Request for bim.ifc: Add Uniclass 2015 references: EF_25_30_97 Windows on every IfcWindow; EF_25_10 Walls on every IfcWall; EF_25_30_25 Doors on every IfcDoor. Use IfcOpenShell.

First a look at what the model holds.

```python
import ifcopenshell

model = ifcopenshell.open("bim.ifc")
print(model.schema)
print("classifications:", [c.Name for c in model.by_type("IfcClassification")])
for ifc_class in ("IfcDoor", "IfcRoof", "IfcStair", "IfcWall", "IfcWindow"):
    print(ifc_class, len(model.by_type(ifc_class)))
```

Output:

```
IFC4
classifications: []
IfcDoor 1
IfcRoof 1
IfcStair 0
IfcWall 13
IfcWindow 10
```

```python
import ifcopenshell
import ifcopenshell.api.classification

model = ifcopenshell.open("bim.ifc")

system = ifcopenshell.api.classification.add_classification(model, classification="Uniclass 2015")

codes = {
    "IfcWindow": ("EF_25_30_97", "Windows"),
    "IfcWall": ("EF_25_10", "Walls"),
    "IfcDoor": ("EF_25_30_25", "Doors"),
}
for ifc_class, (code, name) in codes.items():
    products = model.by_type(ifc_class)
    ifcopenshell.api.classification.add_reference(
        model, products=products, classification=system, identification=code, name=name
    )
    print(code, len(products))

model.write("bim-out.ifc")
```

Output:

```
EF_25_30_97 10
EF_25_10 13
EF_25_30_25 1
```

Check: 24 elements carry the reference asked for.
